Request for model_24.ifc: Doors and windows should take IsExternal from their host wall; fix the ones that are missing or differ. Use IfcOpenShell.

First a look at what the model holds.

```python
import ifcopenshell
import ifcopenshell.util.element

model = ifcopenshell.open("model_24.ifc")
print(model.schema)
seen = {}
for e in model.by_type("IfcDoor") + model.by_type("IfcWindow"):
    if not e.FillsVoids:
        continue
    host = e.FillsVoids[0].RelatingOpeningElement.VoidsElements[0].RelatingBuildingElement
    own = ifcopenshell.util.element.get_pset(e, f"Pset_{e.is_a()[3:].removesuffix('StandardCase')}Common", "IsExternal")
    wall = ifcopenshell.util.element.get_pset(host, "Pset_WallCommon", "IsExternal")
    seen[e.is_a(), own, wall] = seen.get((e.is_a(), own, wall), 0) + 1
for (cls, own, wall), count in sorted(seen.items(), key=str):
    print(count, cls, "IsExternal:", own, "| host wall:", wall)
```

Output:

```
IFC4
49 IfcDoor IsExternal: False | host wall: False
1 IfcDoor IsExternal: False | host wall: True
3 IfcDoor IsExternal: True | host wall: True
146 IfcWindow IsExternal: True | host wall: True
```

```python
import ifcopenshell
import ifcopenshell.api.pset
import ifcopenshell.util.element

model = ifcopenshell.open("model_24.ifc")

count = 0
for ifc_class, pset_name in (("IfcDoor", "Pset_DoorCommon"), ("IfcWindow", "Pset_WindowCommon")):
    for e in model.by_type(ifc_class):
        if not e.FillsVoids:
            continue
        host = e.FillsVoids[0].RelatingOpeningElement.VoidsElements[0].RelatingBuildingElement
        external = ifcopenshell.util.element.get_pset(host, "Pset_WallCommon", "IsExternal")
        if external is None or ifcopenshell.util.element.get_pset(e, pset_name, "IsExternal") == external:
            continue
        pset = ifcopenshell.api.pset.add_pset(model, product=e, name=pset_name)
        ifcopenshell.api.pset.edit_pset(model, pset=pset, properties={"IsExternal": external})
        count += 1

print(count, "updated")

model.write("model_24-out.ifc")
```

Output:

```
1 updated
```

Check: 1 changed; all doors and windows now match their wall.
